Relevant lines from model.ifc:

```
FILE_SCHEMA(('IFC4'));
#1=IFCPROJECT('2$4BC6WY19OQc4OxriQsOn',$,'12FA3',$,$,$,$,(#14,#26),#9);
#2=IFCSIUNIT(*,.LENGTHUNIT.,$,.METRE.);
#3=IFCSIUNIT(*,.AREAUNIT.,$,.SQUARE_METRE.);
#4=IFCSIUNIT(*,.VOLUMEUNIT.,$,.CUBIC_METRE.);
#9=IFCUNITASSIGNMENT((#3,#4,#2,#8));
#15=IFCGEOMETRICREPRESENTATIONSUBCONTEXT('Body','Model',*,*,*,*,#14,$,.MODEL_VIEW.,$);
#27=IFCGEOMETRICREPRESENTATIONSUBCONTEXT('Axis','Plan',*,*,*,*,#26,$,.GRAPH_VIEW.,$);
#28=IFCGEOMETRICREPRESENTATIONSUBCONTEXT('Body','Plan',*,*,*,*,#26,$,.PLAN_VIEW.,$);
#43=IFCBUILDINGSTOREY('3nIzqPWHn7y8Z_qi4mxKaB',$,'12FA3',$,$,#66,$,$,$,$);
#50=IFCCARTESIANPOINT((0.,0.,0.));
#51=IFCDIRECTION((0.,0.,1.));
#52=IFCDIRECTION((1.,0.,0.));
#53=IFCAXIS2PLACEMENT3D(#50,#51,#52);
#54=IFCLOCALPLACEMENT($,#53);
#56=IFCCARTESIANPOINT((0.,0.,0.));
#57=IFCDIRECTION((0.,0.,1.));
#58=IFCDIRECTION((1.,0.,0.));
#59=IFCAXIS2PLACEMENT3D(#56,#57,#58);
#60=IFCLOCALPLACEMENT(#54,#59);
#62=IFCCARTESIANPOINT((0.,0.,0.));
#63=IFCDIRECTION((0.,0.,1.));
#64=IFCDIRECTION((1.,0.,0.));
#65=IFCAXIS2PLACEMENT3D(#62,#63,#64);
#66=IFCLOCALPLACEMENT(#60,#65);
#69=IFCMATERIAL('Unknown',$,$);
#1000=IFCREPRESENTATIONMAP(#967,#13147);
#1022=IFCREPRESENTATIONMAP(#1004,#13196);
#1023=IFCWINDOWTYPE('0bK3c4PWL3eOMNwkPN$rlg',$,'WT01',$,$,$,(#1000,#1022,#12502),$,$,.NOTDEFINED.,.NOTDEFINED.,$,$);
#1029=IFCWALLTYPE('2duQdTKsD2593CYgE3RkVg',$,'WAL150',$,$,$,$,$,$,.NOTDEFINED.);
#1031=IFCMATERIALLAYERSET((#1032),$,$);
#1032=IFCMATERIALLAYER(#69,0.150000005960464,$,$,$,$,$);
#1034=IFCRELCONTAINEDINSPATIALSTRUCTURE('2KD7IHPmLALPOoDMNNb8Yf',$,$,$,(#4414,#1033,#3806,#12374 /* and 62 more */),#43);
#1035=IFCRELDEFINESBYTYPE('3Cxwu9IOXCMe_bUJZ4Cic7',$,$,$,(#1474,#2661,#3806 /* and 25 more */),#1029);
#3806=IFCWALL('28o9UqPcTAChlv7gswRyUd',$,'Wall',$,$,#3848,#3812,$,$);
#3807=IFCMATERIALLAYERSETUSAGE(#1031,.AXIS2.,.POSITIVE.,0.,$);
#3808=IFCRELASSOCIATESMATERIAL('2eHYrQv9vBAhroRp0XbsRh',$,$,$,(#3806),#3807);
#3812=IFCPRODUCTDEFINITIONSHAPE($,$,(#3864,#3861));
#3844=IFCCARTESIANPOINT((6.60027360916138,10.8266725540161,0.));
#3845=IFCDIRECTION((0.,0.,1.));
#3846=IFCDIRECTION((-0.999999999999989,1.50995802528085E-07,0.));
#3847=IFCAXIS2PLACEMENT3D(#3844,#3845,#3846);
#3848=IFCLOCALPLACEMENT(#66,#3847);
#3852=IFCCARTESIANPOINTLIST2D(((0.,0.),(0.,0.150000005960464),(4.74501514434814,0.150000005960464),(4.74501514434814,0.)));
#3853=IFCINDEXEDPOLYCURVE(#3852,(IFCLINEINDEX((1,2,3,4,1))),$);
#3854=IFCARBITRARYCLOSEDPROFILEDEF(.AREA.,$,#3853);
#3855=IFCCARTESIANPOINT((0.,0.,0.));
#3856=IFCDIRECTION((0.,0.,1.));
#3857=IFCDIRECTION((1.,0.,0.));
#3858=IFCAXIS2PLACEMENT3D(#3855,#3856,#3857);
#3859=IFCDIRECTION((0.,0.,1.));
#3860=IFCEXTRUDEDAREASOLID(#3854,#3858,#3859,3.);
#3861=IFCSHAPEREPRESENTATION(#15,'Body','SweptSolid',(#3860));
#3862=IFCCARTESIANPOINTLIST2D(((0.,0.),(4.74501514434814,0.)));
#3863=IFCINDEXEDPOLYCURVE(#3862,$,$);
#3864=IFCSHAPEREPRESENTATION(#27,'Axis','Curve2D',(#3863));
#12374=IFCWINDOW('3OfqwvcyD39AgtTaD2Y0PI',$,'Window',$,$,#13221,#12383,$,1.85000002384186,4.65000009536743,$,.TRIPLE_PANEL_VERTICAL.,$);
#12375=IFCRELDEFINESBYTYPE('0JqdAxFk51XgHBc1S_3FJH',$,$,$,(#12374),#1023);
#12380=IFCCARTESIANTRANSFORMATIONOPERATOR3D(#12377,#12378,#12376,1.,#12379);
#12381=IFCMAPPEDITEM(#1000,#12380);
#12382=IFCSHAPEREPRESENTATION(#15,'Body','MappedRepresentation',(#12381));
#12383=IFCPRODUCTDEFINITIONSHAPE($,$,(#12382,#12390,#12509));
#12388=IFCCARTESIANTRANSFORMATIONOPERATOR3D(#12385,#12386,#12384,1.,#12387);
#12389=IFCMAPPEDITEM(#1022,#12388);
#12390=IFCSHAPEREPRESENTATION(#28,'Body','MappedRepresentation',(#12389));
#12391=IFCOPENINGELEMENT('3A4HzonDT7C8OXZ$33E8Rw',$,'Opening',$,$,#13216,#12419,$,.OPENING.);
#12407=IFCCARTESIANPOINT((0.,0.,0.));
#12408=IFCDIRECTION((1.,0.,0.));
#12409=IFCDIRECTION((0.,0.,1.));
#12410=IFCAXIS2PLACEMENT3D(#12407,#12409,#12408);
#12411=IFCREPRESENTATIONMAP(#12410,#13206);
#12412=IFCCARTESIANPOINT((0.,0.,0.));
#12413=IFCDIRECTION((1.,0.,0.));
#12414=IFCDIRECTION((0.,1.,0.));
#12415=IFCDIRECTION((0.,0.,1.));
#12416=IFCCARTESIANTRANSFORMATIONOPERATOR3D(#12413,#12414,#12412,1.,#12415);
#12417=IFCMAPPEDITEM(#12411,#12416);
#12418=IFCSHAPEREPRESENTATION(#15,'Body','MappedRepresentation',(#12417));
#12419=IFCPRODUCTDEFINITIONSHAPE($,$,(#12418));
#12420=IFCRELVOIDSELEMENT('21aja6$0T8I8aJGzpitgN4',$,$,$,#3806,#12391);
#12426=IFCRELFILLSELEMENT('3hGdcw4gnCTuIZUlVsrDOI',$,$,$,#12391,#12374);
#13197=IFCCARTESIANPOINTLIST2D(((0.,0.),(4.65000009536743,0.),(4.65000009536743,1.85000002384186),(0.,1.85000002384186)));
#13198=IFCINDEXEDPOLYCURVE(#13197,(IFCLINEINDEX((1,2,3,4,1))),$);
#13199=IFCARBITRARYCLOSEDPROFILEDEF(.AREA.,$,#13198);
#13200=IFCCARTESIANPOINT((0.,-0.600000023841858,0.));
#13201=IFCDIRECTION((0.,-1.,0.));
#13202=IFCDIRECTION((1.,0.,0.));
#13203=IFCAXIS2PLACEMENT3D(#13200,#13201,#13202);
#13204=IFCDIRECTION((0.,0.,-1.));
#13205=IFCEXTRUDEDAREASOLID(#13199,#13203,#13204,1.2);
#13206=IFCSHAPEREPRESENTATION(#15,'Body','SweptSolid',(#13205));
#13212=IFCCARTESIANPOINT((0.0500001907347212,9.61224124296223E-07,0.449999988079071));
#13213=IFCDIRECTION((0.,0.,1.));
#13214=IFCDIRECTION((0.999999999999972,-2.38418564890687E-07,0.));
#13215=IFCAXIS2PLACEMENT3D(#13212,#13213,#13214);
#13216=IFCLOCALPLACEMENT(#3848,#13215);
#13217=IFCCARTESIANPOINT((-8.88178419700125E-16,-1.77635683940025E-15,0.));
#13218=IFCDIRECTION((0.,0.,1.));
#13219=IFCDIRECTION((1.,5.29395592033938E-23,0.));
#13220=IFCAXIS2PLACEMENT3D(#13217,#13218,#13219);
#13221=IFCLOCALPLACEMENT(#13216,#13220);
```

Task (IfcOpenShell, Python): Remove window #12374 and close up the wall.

```python
import ifcopenshell
import ifcopenshell.api.feature
import ifcopenshell.api.root
import ifcopenshell.geom
import ifcopenshell.util.shape

model = ifcopenshell.open("model.ifc")
settings = ifcopenshell.geom.settings()


def volume(element):
    """Net volume in cubic metres, openings subtracted."""
    shape = ifcopenshell.geom.create_shape(settings, element)
    return ifcopenshell.util.shape.get_volume(shape.geometry)


window = model.by_guid("3OfqwvcyD39AgtTaD2Y0PI")
opening = window.FillsVoids[0].RelatingOpeningElement
wall = opening.VoidsElements[0].RelatingBuildingElement
before = volume(wall)

ifcopenshell.api.root.remove_product(model, product=window)
ifcopenshell.api.feature.remove_feature(model, feature=opening)

after = volume(wall)

print(f"wall volume {before:.3f} -> {after:.3f} m3")

model.write("model_edited.ifc")
```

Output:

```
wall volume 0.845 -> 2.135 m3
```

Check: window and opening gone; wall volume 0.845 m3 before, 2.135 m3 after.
